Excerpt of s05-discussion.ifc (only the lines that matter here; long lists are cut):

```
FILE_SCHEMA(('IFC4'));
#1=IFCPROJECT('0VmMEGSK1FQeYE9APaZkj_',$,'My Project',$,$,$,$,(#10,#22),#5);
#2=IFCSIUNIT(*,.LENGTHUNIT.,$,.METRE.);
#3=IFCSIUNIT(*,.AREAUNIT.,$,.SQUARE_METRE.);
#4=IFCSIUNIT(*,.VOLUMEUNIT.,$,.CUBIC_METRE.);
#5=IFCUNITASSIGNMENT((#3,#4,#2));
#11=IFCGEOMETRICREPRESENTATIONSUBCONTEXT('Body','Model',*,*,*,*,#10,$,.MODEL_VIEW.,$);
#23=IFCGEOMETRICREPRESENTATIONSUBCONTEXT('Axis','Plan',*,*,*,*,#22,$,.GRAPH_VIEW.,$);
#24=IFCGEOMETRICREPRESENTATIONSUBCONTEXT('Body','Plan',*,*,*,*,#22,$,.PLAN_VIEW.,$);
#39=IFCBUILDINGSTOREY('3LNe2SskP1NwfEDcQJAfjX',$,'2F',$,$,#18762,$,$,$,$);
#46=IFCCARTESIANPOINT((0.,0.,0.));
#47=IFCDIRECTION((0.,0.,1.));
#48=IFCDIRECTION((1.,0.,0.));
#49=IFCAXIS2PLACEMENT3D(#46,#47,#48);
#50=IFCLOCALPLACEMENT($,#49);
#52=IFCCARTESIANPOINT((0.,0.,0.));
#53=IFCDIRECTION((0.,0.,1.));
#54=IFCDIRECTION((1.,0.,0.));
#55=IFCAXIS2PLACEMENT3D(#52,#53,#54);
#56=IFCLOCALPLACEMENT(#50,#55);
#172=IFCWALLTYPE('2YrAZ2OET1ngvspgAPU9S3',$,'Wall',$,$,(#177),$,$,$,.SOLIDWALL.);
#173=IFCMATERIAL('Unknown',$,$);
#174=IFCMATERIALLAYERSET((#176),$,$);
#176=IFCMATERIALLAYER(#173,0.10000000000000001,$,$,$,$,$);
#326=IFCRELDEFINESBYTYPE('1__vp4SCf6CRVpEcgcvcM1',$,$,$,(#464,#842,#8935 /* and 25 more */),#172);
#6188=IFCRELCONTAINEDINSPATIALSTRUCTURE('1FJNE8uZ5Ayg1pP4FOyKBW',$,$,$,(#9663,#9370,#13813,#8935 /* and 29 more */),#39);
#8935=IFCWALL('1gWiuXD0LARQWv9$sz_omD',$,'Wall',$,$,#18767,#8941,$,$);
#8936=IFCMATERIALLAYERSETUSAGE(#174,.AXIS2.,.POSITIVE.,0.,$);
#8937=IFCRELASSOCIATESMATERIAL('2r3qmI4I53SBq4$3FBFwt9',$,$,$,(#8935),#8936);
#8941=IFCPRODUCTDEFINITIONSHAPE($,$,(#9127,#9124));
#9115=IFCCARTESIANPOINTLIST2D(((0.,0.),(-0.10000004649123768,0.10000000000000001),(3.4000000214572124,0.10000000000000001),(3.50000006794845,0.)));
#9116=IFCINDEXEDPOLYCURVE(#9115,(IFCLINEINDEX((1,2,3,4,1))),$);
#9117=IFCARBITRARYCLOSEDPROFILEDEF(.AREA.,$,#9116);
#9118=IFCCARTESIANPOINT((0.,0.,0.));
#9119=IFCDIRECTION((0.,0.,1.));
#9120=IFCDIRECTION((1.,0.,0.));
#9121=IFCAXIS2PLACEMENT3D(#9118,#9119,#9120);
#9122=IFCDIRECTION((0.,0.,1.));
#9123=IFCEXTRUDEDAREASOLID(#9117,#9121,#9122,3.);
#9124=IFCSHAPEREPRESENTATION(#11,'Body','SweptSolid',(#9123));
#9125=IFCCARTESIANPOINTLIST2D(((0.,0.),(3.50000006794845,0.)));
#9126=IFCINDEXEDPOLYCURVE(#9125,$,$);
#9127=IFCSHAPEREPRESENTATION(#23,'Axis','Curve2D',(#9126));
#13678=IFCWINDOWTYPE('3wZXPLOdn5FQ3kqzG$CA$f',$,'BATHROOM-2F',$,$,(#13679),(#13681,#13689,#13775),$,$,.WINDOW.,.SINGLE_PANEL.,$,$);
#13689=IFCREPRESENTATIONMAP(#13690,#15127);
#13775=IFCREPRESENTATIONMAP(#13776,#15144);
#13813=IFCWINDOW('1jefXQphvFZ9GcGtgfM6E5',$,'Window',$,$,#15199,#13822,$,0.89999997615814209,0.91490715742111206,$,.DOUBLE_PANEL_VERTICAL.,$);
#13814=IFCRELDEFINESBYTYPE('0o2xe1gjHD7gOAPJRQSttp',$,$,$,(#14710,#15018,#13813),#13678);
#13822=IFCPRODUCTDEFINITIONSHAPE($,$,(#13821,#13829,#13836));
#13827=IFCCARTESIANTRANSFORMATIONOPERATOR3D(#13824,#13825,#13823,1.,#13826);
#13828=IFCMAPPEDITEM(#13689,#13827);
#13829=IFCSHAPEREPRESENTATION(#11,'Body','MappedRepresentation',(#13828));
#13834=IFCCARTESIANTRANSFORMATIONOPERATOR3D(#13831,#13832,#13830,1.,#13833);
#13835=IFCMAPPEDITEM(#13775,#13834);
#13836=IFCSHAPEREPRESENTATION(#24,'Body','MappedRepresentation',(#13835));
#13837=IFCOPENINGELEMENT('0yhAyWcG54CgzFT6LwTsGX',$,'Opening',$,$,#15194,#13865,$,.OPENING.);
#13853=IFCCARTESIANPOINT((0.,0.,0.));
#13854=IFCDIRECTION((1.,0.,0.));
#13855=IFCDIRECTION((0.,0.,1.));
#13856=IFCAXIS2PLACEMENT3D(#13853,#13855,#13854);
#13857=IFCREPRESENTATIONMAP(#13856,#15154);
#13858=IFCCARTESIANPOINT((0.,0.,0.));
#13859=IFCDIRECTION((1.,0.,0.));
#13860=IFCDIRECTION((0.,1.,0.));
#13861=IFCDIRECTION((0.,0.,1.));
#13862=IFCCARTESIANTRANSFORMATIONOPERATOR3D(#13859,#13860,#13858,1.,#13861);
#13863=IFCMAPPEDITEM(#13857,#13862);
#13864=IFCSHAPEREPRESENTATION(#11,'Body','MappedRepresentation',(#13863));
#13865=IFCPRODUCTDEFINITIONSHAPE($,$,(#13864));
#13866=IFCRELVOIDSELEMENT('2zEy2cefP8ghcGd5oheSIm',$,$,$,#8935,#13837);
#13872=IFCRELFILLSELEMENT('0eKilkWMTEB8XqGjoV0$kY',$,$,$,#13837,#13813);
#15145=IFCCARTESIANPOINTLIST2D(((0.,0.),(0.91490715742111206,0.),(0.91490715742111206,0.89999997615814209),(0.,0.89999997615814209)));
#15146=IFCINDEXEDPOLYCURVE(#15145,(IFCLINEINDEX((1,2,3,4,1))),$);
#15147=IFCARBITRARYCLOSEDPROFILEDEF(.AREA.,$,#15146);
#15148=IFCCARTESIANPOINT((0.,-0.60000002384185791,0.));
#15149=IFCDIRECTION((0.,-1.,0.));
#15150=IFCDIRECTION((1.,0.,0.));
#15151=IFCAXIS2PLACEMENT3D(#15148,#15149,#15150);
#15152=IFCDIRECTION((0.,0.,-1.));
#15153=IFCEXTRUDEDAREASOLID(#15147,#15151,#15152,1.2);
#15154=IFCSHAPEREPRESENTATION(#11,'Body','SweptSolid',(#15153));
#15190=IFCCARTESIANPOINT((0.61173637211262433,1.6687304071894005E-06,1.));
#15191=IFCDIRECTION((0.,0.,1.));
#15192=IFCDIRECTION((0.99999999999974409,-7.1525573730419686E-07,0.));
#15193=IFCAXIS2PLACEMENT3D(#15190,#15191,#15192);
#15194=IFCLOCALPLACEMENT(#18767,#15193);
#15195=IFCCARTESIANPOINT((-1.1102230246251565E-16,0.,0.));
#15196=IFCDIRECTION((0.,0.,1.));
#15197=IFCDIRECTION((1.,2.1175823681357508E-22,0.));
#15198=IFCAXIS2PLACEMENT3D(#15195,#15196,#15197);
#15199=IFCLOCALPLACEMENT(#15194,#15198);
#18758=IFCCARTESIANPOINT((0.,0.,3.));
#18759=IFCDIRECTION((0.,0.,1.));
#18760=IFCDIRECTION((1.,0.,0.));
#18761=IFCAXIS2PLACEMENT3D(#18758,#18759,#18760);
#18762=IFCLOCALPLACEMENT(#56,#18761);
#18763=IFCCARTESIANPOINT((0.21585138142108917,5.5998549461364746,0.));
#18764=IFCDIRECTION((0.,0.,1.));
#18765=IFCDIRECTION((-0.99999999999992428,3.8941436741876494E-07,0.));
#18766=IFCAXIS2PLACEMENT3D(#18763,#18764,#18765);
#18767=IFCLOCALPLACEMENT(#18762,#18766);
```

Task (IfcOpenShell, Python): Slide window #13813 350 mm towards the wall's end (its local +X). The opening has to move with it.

```python
import ifcopenshell
import ifcopenshell.api.geometry
import ifcopenshell.util.placement

model = ifcopenshell.open("s05-discussion.ifc")

window = model.by_id(13813)
opening = window.FillsVoids[0].RelatingOpeningElement
wall = opening.VoidsElements[0].RelatingBuildingElement

wall_matrix = ifcopenshell.util.placement.get_local_placement(wall.ObjectPlacement)
shift = wall_matrix[:3, 0] * 0.35
before = ifcopenshell.util.placement.get_local_placement(window.ObjectPlacement)[:3, 3].copy()

# The window is placed relative to its opening, so it follows when the opening moves.
matrix = ifcopenshell.util.placement.get_local_placement(opening.ObjectPlacement)
matrix[:3, 3] += shift
ifcopenshell.api.geometry.edit_object_placement(
    model, product=opening, matrix=matrix, is_si=False, should_transform_children=True
)

after = ifcopenshell.util.placement.get_local_placement(window.ObjectPlacement)[:3, 3]
print("window moved by", (after - before).round(3) + 0.0)

model.write("s05-discussion_edited.ifc")
```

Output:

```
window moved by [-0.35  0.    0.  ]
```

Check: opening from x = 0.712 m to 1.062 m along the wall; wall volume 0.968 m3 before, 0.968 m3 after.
